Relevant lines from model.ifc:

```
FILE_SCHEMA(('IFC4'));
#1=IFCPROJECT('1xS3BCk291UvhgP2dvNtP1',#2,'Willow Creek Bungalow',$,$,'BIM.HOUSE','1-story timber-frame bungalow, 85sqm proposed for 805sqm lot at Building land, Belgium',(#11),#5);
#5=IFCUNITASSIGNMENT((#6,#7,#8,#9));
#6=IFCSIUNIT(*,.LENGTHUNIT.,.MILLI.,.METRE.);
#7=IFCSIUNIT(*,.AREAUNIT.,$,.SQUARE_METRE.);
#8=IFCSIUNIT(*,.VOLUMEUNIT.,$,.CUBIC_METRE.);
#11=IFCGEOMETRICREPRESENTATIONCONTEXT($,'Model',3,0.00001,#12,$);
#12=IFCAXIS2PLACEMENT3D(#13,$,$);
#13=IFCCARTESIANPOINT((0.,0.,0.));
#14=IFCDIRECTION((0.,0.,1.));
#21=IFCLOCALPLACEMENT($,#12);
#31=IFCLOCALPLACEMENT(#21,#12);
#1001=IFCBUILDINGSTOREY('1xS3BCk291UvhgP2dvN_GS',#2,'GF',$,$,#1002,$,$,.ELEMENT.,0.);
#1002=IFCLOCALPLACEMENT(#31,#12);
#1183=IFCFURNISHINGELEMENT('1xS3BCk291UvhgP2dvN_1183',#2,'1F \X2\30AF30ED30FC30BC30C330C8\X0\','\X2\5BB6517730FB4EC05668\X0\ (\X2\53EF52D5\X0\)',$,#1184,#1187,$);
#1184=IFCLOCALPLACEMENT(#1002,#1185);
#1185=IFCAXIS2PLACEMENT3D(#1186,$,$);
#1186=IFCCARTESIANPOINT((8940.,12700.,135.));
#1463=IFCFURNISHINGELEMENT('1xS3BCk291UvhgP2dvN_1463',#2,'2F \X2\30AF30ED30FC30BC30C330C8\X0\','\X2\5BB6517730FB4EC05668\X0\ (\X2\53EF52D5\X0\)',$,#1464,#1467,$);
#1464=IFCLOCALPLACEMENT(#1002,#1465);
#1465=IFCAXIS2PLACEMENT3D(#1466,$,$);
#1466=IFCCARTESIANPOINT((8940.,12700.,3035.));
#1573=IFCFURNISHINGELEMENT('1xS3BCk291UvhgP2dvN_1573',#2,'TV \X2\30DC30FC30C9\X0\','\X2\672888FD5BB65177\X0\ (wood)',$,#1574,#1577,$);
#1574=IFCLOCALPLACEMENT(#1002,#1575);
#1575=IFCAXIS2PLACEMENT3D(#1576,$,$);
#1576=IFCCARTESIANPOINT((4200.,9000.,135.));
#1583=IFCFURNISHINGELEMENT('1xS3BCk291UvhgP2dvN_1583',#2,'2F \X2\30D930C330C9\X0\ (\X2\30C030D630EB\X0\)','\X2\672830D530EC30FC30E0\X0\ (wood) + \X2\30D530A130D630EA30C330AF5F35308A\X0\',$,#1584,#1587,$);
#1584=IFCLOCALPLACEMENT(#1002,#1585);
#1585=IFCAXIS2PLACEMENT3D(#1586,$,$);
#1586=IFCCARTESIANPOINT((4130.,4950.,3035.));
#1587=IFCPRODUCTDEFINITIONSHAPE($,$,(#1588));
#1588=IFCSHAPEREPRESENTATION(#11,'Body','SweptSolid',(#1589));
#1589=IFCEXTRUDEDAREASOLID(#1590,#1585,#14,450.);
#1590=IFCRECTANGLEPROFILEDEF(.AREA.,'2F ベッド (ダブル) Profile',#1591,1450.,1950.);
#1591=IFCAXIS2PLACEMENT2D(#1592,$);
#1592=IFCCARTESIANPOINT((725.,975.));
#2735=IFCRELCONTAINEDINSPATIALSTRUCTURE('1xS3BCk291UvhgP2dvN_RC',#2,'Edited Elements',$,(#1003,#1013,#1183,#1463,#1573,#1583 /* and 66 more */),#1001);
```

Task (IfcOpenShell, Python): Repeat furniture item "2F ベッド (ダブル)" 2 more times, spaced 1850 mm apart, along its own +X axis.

```python
import ifcopenshell
import ifcopenshell.api.geometry
import ifcopenshell.api.root
import ifcopenshell.util.element
import ifcopenshell.util.placement
import ifcopenshell.util.unit

model = ifcopenshell.open("model.ifc")
unit_scale = ifcopenshell.util.unit.calculate_unit_scale(model)


def reuse_history(source, copy):
    """copy_class also copies each property set's owner history, people and application; keep the originals."""
    for rel in copy.IsDefinedBy:
        if rel.is_a("IfcRelDefinesByProperties") and (history := rel.RelatingPropertyDefinition.OwnerHistory):
            rel.RelatingPropertyDefinition.OwnerHistory = source.OwnerHistory
            ifcopenshell.util.element.remove_deep2(model, history)


source = model.by_guid("1xS3BCk291UvhgP2dvN_1583")
base = ifcopenshell.util.placement.get_local_placement(source.ObjectPlacement)
step = base[:3, 0] * 1.85 / unit_scale

for i in range(1, 3):
    copy = ifcopenshell.api.root.copy_class(model, product=source)
    copy.Representation = ifcopenshell.util.element.copy_deep(
        model, source.Representation, exclude=["IfcGeometricRepresentationContext", "IfcRepresentationMap"]
    )
    reuse_history(source, copy)
    matrix = base.copy()
    matrix[:3, 3] += i * step
    print("added at", matrix[:3, 3].round(3) + 0.0)
    ifcopenshell.api.geometry.edit_object_placement(model, product=copy, matrix=matrix, is_si=False)

model.write("model_v2.ifc")
```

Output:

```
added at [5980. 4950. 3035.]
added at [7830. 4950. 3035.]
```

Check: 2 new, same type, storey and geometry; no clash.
